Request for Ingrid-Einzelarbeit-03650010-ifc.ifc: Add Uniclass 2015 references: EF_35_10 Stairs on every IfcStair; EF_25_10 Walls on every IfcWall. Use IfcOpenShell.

First a look at what the model holds.

```python
import ifcopenshell

model = ifcopenshell.open("Ingrid-Einzelarbeit-03650010-ifc.ifc")
print(model.schema)
print("classifications:", [c.Name for c in model.by_type("IfcClassification")])
for ifc_class in ("IfcDoor", "IfcRoof", "IfcStair", "IfcWall", "IfcWindow"):
    print(ifc_class, len(model.by_type(ifc_class)))
```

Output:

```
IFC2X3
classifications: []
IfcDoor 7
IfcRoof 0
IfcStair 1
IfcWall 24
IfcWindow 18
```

```python
import ifcopenshell
import ifcopenshell.api.classification

model = ifcopenshell.open("Ingrid-Einzelarbeit-03650010-ifc.ifc")

# IFC2X3 requires Source and Edition and has no link from the project to the system.
system = model.create_entity("IfcClassification", Source="NBS", Edition="2015", Name="Uniclass 2015")

codes = {
    "IfcStair": ("EF_35_10", "Stairs"),
    "IfcWall": ("EF_25_10", "Walls"),
}
for ifc_class, (code, name) in codes.items():
    products = model.by_type(ifc_class)
    ifcopenshell.api.classification.add_reference(
        model, products=products, classification=system, identification=code, name=name
    )
    print(code, len(products))

model.write("Ingrid-Einzelarbeit-03650010-ifc_v2.ifc")
```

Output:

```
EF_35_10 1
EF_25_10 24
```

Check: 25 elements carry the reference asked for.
